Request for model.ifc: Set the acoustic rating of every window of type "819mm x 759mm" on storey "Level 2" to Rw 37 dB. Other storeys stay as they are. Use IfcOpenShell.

First a look at what the model holds.

```python
import ifcopenshell
import ifcopenshell.util.element

model = ifcopenshell.open("model.ifc")
print(model.schema)
storey = next(s for s in model.by_type("IfcBuildingStorey") if s.Name == "Level 2")
windows = [e for e in ifcopenshell.util.element.get_decomposition(storey) if e.is_a("IfcWindow")]
seen = {}
for e in windows:
    element_type = ifcopenshell.util.element.get_type(e)
    key = (element_type.Name if element_type != e and element_type else None, ifcopenshell.util.element.get_pset(e, "Pset_WindowCommon", "AcousticRating"))
    seen[key] = seen.get(key, 0) + 1
for (name, value), count in sorted(seen.items(), key=str):
    print(count, "x", name, "|", value)
```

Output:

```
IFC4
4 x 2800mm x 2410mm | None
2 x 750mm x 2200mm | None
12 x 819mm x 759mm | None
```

```python
import ifcopenshell
import ifcopenshell.api.pset
import ifcopenshell.util.element

model = ifcopenshell.open("model.ifc")

storey = next(s for s in model.by_type("IfcBuildingStorey") if s.Name == "Level 2")
windows = [e for e in ifcopenshell.util.element.get_decomposition(storey) if e.is_a("IfcWindow")]

count = 0
for e in windows:
    element_type = ifcopenshell.util.element.get_type(e)
    if element_type in (None, e) or element_type.Name != "819mm x 759mm":
        continue
    # add_pset returns the element's existing set when there is one.
    pset = ifcopenshell.api.pset.add_pset(model, product=e, name="Pset_WindowCommon")
    ifcopenshell.api.pset.edit_pset(model, pset=pset, properties={"AcousticRating": "Rw 37 dB"})
    count += 1

print(count, "windows updated")

model.write("model_updated.ifc")
```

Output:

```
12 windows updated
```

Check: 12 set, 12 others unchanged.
